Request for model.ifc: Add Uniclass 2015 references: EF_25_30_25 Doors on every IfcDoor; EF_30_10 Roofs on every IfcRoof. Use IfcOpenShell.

First a look at what the model holds.

```python
import ifcopenshell

model = ifcopenshell.open("model.ifc")
print(model.schema)
print("classifications:", [c.Name for c in model.by_type("IfcClassification")])
for ifc_class in ("IfcDoor", "IfcRoof", "IfcStair", "IfcWall", "IfcWindow"):
    print(ifc_class, len(model.by_type(ifc_class)))
```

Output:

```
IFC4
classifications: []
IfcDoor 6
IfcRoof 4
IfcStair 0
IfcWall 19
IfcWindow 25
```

```python
import ifcopenshell
import ifcopenshell.api.classification

model = ifcopenshell.open("model.ifc")

system = ifcopenshell.api.classification.add_classification(model, classification="Uniclass 2015")

codes = {
    "IfcDoor": ("EF_25_30_25", "Doors"),
    "IfcRoof": ("EF_30_10", "Roofs"),
}
for ifc_class, (code, name) in codes.items():
    products = model.by_type(ifc_class)
    ifcopenshell.api.classification.add_reference(
        model, products=products, classification=system, identification=code, name=name
    )
    print(code, len(products))

model.write("model_v2.ifc")
```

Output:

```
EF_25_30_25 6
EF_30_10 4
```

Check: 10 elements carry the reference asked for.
